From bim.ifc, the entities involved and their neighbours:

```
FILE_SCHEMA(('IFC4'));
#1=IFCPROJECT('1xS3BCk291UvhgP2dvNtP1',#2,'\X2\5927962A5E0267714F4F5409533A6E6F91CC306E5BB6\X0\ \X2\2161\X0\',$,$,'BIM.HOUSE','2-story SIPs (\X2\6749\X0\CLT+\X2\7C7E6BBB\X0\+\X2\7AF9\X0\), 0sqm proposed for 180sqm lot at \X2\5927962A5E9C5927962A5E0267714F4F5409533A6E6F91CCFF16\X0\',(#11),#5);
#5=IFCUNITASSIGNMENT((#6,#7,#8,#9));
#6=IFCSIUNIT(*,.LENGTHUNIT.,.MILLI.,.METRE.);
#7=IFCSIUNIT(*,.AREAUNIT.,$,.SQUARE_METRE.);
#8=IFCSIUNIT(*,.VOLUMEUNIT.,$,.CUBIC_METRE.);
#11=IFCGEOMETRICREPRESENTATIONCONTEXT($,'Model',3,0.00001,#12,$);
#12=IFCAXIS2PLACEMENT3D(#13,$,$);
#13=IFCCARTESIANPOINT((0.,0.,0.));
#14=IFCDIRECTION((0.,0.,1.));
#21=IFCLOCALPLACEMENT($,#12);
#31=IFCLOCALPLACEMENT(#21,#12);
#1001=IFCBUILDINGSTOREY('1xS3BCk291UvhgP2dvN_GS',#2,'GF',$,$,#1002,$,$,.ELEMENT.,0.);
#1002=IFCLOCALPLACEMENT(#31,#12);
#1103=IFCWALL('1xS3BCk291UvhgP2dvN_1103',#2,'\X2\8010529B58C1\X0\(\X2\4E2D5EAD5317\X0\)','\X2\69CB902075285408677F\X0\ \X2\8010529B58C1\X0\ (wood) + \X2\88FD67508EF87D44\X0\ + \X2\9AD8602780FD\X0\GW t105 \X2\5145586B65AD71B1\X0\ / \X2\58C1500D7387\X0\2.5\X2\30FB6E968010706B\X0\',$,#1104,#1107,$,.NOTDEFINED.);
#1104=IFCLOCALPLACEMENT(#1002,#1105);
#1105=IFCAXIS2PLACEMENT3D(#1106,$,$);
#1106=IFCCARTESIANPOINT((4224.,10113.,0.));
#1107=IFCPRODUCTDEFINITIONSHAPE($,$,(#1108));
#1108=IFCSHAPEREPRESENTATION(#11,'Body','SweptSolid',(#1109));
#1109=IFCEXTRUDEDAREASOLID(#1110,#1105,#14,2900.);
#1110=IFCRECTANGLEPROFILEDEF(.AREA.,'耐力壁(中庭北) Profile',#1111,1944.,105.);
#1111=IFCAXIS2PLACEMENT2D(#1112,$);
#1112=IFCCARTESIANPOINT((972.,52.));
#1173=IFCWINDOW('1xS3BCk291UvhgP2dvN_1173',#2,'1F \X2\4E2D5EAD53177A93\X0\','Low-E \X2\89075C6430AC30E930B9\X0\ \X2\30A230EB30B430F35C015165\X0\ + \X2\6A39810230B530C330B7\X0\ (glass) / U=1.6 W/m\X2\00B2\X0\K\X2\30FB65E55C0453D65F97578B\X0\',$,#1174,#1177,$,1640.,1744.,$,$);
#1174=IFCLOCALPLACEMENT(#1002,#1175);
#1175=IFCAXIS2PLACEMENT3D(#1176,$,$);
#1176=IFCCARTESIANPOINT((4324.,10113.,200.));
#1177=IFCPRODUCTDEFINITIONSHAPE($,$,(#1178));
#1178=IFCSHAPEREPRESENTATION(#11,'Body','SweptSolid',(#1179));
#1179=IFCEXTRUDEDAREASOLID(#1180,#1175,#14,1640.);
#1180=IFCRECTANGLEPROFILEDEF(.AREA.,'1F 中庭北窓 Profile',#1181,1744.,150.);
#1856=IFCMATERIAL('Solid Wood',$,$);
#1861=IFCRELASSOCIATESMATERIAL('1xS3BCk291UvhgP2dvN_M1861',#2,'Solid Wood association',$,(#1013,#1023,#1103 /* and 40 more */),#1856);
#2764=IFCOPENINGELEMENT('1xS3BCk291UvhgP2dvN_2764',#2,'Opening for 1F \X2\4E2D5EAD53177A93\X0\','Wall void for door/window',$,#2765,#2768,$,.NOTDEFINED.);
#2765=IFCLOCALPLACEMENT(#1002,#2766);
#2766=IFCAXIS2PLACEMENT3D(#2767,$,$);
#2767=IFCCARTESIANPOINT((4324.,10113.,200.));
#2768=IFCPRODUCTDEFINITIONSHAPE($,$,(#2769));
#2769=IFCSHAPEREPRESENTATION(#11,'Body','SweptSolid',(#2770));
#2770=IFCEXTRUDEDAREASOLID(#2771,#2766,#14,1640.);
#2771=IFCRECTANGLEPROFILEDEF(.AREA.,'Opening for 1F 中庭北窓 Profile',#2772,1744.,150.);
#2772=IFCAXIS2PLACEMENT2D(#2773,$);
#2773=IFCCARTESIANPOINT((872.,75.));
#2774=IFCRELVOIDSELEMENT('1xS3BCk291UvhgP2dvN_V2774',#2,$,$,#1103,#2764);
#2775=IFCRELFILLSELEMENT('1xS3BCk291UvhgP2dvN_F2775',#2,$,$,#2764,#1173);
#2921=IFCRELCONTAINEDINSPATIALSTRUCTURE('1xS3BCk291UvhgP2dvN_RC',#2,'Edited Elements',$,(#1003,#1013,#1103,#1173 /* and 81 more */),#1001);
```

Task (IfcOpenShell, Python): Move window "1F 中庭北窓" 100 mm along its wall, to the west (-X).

```python
import ifcopenshell
import ifcopenshell.api.geometry
import ifcopenshell.util.placement
import ifcopenshell.util.unit

model = ifcopenshell.open("bim.ifc")
unit_scale = ifcopenshell.util.unit.calculate_unit_scale(model)

window = model.by_id(1173)
opening = window.FillsVoids[0].RelatingOpeningElement
wall = opening.VoidsElements[0].RelatingBuildingElement

wall_matrix = ifcopenshell.util.placement.get_local_placement(wall.ObjectPlacement)
shift = wall_matrix[:3, 0] * -0.1 / unit_scale
before = ifcopenshell.util.placement.get_local_placement(window.ObjectPlacement)[:3, 3].copy()

# The window is not placed relative to its opening, so move both.
for product in (opening, window):
    matrix = ifcopenshell.util.placement.get_local_placement(product.ObjectPlacement)
    matrix[:3, 3] += shift
    ifcopenshell.api.geometry.edit_object_placement(model, product=product, matrix=matrix, is_si=False)

after = ifcopenshell.util.placement.get_local_placement(window.ObjectPlacement)[:3, 3]
print("window moved by", (after - before).round(3) + 0.0)

model.write("bim_updated.ifc")
```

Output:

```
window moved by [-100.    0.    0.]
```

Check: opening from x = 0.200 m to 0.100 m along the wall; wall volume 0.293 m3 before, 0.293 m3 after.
